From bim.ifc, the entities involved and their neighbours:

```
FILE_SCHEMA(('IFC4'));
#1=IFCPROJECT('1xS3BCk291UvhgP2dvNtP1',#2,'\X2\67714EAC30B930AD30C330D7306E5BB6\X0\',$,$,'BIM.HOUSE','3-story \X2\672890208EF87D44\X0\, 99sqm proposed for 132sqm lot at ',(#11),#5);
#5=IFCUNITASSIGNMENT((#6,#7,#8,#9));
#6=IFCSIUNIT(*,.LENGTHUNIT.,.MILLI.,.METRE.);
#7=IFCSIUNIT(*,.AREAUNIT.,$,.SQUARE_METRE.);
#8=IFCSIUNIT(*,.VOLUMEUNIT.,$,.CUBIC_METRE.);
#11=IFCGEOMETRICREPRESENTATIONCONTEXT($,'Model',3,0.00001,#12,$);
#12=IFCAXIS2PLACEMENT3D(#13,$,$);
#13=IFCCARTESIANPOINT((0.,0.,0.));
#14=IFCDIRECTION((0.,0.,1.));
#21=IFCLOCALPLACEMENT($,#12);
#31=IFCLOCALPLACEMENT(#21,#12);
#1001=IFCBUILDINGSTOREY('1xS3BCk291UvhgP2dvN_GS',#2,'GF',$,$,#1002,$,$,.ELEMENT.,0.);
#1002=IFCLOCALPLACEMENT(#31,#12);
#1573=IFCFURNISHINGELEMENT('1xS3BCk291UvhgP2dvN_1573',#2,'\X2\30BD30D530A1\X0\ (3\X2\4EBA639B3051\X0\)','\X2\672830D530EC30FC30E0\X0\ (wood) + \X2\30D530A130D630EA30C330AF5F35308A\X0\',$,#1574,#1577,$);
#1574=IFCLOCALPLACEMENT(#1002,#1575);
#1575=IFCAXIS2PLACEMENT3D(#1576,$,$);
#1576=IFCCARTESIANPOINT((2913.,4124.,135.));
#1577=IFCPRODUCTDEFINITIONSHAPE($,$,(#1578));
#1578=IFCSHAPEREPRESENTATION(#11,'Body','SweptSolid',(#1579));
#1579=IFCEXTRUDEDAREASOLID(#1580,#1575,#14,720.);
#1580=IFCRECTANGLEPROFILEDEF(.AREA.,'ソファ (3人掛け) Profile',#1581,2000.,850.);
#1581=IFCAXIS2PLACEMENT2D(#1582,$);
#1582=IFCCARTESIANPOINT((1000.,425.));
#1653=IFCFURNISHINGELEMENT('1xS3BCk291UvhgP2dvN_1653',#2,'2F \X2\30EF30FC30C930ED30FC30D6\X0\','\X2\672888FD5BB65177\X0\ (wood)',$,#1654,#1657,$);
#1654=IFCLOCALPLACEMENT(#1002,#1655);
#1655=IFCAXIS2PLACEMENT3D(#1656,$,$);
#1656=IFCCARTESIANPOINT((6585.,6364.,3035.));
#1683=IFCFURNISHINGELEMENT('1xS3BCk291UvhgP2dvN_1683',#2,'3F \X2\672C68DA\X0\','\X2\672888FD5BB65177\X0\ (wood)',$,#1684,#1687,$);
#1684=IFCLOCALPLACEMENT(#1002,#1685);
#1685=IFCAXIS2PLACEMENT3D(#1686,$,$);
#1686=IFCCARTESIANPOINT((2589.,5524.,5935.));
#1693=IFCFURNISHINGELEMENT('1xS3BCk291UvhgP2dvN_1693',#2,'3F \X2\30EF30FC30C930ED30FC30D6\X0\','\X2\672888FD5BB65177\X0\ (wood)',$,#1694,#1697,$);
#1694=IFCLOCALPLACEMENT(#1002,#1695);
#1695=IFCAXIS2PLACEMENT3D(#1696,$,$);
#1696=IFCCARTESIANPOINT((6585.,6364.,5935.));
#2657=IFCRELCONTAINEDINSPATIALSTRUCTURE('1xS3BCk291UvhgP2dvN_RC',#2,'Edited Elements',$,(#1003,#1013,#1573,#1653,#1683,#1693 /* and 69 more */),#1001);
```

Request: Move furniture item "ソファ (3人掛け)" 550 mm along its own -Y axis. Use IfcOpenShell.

```python
import ifcopenshell
import ifcopenshell.api.geometry
import ifcopenshell.util.placement
import ifcopenshell.util.unit

model = ifcopenshell.open("bim.ifc")
unit_scale = ifcopenshell.util.unit.calculate_unit_scale(model)

item = model.by_guid("1xS3BCk291UvhgP2dvN_1573")
matrix = ifcopenshell.util.placement.get_local_placement(item.ObjectPlacement)
matrix[:3, 3] -= matrix[:3, 1] * 0.55 / unit_scale
ifcopenshell.api.geometry.edit_object_placement(model, product=item, matrix=matrix, is_si=False)

print(ifcopenshell.util.placement.get_local_placement(item.ObjectPlacement).round(3) + 0.0)

model.write("bim_v2.ifc")
```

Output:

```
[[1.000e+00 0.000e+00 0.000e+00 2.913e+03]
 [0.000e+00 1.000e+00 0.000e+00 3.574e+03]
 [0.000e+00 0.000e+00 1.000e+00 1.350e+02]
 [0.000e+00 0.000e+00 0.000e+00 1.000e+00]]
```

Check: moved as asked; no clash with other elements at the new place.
